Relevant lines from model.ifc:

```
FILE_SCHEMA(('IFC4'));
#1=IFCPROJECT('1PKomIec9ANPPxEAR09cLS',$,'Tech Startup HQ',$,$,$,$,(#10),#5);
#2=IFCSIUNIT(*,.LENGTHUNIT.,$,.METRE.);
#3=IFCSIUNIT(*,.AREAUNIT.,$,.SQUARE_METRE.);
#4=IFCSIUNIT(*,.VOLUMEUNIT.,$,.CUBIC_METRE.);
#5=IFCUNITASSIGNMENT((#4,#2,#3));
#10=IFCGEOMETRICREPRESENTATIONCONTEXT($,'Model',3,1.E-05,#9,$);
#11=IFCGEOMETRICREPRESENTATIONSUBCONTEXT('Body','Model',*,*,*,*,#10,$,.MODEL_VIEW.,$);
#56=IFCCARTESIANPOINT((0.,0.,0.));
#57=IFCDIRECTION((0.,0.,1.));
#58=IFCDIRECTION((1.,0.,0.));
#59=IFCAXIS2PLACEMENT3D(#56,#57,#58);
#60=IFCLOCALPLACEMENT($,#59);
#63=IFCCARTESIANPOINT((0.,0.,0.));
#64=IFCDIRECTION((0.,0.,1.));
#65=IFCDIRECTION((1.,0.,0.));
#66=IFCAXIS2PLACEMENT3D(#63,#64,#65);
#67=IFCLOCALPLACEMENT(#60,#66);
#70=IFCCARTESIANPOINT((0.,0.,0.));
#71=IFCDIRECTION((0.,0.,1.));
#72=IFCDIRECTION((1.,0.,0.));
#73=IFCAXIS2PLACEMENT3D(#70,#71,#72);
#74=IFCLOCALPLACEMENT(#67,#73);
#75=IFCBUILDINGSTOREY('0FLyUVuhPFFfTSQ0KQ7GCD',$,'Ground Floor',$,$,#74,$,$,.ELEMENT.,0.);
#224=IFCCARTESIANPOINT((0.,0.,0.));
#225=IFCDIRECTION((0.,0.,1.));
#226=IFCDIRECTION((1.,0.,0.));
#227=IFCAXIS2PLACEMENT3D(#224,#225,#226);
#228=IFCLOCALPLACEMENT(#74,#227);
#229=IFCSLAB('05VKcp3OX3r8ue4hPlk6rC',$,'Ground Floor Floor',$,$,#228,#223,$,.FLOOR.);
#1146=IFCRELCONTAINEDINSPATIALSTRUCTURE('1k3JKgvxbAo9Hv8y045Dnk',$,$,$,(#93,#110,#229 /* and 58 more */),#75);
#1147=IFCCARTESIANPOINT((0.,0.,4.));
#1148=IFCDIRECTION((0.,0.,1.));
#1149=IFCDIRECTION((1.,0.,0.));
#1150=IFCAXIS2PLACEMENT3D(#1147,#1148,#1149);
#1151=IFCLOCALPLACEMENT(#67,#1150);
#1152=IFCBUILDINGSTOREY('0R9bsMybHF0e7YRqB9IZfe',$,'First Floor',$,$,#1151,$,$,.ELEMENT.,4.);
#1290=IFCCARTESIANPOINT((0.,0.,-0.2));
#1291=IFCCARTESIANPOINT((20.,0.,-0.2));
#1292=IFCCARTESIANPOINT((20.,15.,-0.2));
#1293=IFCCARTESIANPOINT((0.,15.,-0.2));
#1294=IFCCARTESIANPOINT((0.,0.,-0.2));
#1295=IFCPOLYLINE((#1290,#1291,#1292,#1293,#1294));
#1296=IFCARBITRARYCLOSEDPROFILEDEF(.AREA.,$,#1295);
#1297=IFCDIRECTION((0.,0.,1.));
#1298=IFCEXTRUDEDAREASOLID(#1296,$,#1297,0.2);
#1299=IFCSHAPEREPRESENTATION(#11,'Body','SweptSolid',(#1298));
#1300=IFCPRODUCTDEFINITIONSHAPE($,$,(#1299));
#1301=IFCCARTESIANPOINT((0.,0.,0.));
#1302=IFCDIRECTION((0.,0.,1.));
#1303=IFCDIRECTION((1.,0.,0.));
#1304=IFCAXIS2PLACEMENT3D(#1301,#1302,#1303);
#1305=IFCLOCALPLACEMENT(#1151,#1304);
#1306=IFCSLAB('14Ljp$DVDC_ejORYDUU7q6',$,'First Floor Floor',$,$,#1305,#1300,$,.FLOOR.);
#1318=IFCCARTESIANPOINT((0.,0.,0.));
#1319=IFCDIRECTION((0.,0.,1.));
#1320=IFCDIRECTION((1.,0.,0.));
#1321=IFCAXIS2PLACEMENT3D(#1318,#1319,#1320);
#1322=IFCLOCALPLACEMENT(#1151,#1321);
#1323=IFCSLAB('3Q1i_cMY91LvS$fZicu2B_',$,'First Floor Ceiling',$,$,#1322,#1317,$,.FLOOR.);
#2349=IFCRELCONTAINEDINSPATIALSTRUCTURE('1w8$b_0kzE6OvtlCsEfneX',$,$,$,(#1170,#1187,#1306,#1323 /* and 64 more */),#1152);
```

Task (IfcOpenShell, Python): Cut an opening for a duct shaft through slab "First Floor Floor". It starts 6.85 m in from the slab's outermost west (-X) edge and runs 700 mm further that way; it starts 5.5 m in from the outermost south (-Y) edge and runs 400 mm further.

```python
import numpy as np
import ifcopenshell
import ifcopenshell.api.feature
import ifcopenshell.api.geometry
import ifcopenshell.api.root
import ifcopenshell.geom
import ifcopenshell.util.placement
import ifcopenshell.util.representation
import ifcopenshell.util.shape
import ifcopenshell.util.unit

model = ifcopenshell.open("model.ifc")
unit_scale = ifcopenshell.util.unit.calculate_unit_scale(model)
settings = ifcopenshell.geom.settings()


def volume(element):
    """Net volume in cubic metres, openings subtracted."""
    shape = ifcopenshell.geom.create_shape(settings, element)
    return ifcopenshell.util.shape.get_volume(shape.geometry)


slab = model.by_guid("14Ljp$DVDC_ejORYDUU7q6")
before = volume(slab)

# Extent in the slab's own axes, in metres. The edges named are its -X and -Y sides.
slab_shape = ifcopenshell.geom.create_shape(settings, slab)
vertices = ifcopenshell.util.shape.get_vertices(slab_shape.geometry)
x_min, y_min, bottom = vertices.min(axis=0)
top = vertices[:, 2].max()

opening = ifcopenshell.api.root.create_entity(model, ifc_class="IfcOpeningElement", name="Duct shaft opening", predefined_type="OPENING")
context = ifcopenshell.util.representation.get_context(model, "Model", "Body", "MODEL_VIEW")
width, depth = 0.7, 0.4
outline = [(0.0, 0.0), (width, 0.0), (width, depth), (0.0, depth), (0.0, 0.0)]
# Overshoot both faces by 50 mm so the cut is clean.
shape = ifcopenshell.api.geometry.add_slab_representation(
    model, context=context, depth=top - bottom + 0.1, polyline=outline
)
ifcopenshell.api.geometry.assign_representation(model, product=opening, representation=shape)

matrix = ifcopenshell.util.placement.get_local_placement(slab.ObjectPlacement)
matrix[:, 3] = matrix @ np.append(np.array([x_min + 6.85, y_min + 5.5, bottom - 0.05]) / unit_scale, 1.0)
ifcopenshell.api.geometry.edit_object_placement(model, product=opening, matrix=matrix, is_si=False)
ifcopenshell.api.feature.add_feature(model, feature=opening, element=slab)

after = volume(slab)

print(f"slab volume {before:.3f} -> {after:.3f} m3")

model.write("model-out.ifc")
```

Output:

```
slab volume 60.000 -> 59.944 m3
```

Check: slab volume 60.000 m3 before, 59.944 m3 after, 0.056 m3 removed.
